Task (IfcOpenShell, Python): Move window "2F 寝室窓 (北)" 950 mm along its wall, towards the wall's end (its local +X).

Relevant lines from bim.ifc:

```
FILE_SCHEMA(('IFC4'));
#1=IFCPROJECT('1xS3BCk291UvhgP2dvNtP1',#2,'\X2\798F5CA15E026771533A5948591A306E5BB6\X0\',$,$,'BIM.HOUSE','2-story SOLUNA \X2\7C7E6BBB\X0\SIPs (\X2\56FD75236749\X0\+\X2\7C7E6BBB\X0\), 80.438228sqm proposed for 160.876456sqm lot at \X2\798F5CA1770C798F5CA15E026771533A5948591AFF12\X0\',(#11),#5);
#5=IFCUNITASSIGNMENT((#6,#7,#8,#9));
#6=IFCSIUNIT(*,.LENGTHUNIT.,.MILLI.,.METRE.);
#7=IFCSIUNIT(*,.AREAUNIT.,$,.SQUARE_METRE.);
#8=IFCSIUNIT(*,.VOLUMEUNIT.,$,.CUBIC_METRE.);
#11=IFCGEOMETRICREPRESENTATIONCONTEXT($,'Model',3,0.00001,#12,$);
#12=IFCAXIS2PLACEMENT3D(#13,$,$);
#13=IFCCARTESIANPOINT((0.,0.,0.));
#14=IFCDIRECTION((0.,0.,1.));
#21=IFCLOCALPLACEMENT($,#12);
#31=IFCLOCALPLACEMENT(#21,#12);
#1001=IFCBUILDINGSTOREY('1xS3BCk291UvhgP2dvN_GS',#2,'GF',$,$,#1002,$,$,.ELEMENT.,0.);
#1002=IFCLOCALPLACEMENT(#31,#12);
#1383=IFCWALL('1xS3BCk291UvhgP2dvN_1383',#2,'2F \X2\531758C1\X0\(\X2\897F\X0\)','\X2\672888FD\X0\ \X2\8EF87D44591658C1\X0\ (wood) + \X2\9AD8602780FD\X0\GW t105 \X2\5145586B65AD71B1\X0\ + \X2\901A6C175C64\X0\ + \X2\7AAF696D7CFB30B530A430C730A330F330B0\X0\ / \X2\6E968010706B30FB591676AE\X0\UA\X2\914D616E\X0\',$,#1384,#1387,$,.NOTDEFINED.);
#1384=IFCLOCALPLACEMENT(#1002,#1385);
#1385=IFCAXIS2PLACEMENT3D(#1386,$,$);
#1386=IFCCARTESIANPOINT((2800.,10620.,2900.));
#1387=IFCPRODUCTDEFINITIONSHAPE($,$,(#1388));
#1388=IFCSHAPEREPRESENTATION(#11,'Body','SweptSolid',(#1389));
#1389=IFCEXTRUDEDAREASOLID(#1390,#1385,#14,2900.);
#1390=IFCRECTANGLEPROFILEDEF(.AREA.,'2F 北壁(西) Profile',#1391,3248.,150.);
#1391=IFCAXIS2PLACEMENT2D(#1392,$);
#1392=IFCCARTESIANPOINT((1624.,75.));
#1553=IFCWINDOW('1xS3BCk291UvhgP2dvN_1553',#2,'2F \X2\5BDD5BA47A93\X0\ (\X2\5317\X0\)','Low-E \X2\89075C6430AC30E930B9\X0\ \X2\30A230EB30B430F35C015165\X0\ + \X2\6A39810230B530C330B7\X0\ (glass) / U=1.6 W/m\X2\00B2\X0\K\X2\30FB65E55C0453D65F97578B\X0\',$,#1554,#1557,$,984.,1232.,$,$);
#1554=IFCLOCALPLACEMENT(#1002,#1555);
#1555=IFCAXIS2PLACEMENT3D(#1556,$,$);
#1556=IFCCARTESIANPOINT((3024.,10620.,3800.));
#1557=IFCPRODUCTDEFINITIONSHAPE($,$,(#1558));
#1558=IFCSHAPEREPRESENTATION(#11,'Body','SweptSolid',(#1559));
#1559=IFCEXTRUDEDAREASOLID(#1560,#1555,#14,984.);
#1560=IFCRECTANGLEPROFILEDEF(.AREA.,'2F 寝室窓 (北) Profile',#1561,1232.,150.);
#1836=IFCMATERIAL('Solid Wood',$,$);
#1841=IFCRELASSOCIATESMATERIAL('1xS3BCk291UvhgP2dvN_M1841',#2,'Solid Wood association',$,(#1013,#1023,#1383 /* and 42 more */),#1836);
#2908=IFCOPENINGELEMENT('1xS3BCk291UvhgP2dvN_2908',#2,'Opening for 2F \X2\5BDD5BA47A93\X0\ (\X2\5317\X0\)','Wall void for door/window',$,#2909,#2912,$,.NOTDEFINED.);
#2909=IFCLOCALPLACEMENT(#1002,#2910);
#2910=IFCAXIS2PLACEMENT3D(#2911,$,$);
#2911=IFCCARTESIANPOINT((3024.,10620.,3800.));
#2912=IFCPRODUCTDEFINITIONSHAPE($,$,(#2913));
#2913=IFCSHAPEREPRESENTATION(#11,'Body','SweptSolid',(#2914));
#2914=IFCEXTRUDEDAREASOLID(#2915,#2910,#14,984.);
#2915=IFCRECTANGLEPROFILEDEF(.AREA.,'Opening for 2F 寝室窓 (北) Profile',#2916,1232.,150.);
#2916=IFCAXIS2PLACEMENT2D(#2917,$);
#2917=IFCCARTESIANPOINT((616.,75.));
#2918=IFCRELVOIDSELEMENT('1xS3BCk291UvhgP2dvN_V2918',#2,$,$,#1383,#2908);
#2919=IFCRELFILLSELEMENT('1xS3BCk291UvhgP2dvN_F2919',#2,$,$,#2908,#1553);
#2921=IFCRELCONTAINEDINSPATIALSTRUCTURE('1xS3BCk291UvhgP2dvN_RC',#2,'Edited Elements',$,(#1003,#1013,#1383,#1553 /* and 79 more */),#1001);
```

```python
import ifcopenshell
import ifcopenshell.api.geometry
import ifcopenshell.util.placement
import ifcopenshell.util.unit

model = ifcopenshell.open("bim.ifc")
unit_scale = ifcopenshell.util.unit.calculate_unit_scale(model)

window = model.by_id(1553)
opening = window.FillsVoids[0].RelatingOpeningElement
wall = opening.VoidsElements[0].RelatingBuildingElement

wall_matrix = ifcopenshell.util.placement.get_local_placement(wall.ObjectPlacement)
shift = wall_matrix[:3, 0] * 0.95 / unit_scale
before = ifcopenshell.util.placement.get_local_placement(window.ObjectPlacement)[:3, 3].copy()

# The window is not placed relative to its opening, so move both.
for product in (opening, window):
    matrix = ifcopenshell.util.placement.get_local_placement(product.ObjectPlacement)
    matrix[:3, 3] += shift
    ifcopenshell.api.geometry.edit_object_placement(model, product=product, matrix=matrix, is_si=False)

after = ifcopenshell.util.placement.get_local_placement(window.ObjectPlacement)[:3, 3]
print("window moved by", (after - before).round(3) + 0.0)

model.write("bim_edited.ifc")
```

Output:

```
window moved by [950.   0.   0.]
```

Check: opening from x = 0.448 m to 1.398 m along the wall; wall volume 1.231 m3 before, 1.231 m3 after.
